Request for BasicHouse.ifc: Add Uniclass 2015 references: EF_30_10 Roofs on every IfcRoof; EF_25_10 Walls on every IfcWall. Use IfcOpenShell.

First a look at what the model holds.

```python
import ifcopenshell

model = ifcopenshell.open("BasicHouse.ifc")
print(model.schema)
print("classifications:", [c.Name for c in model.by_type("IfcClassification")])
for ifc_class in ("IfcDoor", "IfcRoof", "IfcStair", "IfcWall", "IfcWindow"):
    print(ifc_class, len(model.by_type(ifc_class)))
```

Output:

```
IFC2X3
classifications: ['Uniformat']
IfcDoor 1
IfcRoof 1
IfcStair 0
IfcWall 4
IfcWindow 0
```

```python
import ifcopenshell
import ifcopenshell.api.classification

model = ifcopenshell.open("BasicHouse.ifc")

# IFC2X3 requires Source and Edition and has no link from the project to the system.
system = model.create_entity("IfcClassification", Source="NBS", Edition="2015", Name="Uniclass 2015")

codes = {
    "IfcRoof": ("EF_30_10", "Roofs"),
    "IfcWall": ("EF_25_10", "Walls"),
}
for ifc_class, (code, name) in codes.items():
    products = model.by_type(ifc_class)
    ifcopenshell.api.classification.add_reference(
        model, products=products, classification=system, identification=code, name=name
    )
    print(code, len(products))

model.write("BasicHouse_v2.ifc")
```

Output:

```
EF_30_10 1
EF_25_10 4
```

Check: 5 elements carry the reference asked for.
